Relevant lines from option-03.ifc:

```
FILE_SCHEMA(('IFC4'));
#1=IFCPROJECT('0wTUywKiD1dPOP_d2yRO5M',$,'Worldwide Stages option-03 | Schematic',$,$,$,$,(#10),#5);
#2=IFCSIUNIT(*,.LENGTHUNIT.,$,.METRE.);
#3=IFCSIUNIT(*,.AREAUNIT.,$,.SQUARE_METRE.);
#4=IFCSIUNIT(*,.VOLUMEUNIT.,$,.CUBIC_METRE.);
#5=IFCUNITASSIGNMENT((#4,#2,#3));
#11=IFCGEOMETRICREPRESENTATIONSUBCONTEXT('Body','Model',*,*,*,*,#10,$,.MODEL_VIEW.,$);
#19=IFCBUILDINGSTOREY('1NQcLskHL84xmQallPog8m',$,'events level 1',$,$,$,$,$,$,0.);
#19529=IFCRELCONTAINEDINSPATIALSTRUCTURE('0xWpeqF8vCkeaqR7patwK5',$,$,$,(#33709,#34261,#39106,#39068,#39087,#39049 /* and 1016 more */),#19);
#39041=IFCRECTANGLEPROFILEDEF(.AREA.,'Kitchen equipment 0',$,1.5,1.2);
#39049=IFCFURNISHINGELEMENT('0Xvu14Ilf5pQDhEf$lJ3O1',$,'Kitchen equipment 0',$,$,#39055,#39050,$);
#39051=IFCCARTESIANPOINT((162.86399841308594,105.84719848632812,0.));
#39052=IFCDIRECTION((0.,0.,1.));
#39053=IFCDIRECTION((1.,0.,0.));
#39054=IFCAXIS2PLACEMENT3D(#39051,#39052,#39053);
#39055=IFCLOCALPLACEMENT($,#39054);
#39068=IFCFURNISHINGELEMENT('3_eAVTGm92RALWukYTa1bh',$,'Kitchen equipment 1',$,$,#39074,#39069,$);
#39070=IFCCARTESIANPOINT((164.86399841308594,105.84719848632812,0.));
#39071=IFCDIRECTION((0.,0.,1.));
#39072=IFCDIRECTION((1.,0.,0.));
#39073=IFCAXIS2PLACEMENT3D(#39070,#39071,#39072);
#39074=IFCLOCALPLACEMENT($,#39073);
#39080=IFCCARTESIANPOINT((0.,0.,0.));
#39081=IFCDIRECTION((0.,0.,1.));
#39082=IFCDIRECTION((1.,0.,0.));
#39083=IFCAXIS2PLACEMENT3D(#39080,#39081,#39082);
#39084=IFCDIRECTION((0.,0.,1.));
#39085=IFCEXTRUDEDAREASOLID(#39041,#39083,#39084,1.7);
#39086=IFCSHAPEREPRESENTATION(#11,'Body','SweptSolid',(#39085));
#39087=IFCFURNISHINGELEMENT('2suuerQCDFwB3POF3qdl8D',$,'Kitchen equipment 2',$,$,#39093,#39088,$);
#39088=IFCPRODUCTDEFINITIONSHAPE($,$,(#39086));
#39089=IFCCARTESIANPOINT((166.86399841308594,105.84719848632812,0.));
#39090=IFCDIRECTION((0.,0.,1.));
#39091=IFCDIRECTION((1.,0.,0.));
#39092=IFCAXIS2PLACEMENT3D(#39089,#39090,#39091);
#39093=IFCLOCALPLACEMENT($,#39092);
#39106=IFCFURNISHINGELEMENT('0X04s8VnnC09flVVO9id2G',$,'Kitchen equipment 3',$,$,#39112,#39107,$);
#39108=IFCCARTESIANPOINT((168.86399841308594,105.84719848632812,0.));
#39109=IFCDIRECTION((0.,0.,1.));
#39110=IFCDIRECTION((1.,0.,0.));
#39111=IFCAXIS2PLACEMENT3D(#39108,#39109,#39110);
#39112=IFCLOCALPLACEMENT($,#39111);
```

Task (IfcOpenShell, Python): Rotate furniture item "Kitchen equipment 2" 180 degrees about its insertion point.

```python
import ifcopenshell
import ifcopenshell.api.geometry
import ifcopenshell.util.placement

model = ifcopenshell.open("option-03.ifc")

item = model.by_id(39087)
matrix = ifcopenshell.util.placement.get_local_placement(item.ObjectPlacement)
matrix = matrix @ ifcopenshell.util.placement.rotation(180, "Z")
ifcopenshell.api.geometry.edit_object_placement(model, product=item, matrix=matrix, is_si=False)

print(ifcopenshell.util.placement.get_local_placement(item.ObjectPlacement).round(3) + 0.0)

model.write("option-03_edited.ifc")
```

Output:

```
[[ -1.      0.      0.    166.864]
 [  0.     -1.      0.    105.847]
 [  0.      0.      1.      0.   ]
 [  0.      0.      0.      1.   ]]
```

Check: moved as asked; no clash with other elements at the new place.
